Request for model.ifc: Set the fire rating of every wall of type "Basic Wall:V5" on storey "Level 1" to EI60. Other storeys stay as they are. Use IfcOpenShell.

First a look at what the model holds.

```python
import ifcopenshell
import ifcopenshell.util.element

model = ifcopenshell.open("model.ifc")
print(model.schema)
storey = next(s for s in model.by_type("IfcBuildingStorey") if s.Name == "Level 1")
walls = [e for e in ifcopenshell.util.element.get_decomposition(storey) if e.is_a("IfcWall")]
seen = {}
for e in walls:
    element_type = ifcopenshell.util.element.get_type(e)
    key = (element_type.Name if element_type != e and element_type else None, ifcopenshell.util.element.get_pset(e, "Pset_WallCommon", "FireRating"))
    seen[key] = seen.get(key, 0) + 1
for (name, value), count in sorted(seen.items(), key=str):
    print(count, "x", name, "|", value)
```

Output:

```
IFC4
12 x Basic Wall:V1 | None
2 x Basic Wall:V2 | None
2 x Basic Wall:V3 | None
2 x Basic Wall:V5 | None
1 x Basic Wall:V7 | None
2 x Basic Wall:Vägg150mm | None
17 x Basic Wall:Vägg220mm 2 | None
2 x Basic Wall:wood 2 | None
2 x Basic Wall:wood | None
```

```python
import ifcopenshell
import ifcopenshell.api.pset
import ifcopenshell.util.element

model = ifcopenshell.open("model.ifc")

storey = next(s for s in model.by_type("IfcBuildingStorey") if s.Name == "Level 1")
walls = [e for e in ifcopenshell.util.element.get_decomposition(storey) if e.is_a("IfcWall")]

count = 0
for e in walls:
    element_type = ifcopenshell.util.element.get_type(e)
    if element_type in (None, e) or element_type.Name != "Basic Wall:V5":
        continue
    # add_pset returns the element's existing set when there is one.
    pset = ifcopenshell.api.pset.add_pset(model, product=e, name="Pset_WallCommon")
    ifcopenshell.api.pset.edit_pset(model, pset=pset, properties={"FireRating": "EI60"})
    count += 1

print(count, "walls updated")

model.write("model_v2.ifc")
```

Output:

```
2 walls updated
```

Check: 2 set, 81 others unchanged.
